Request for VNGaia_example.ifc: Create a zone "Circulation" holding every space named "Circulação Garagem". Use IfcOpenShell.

First a look at what the model holds.

```python
import ifcopenshell

model = ifcopenshell.open("VNGaia_example.ifc")
print(model.schema)
seen = {}
for space in model.by_type("IfcSpace"):
    seen[space.LongName] = seen.get(space.LongName, 0) + 1
for name, count in sorted(seen.items(), key=str):
    print(count, "x", name)
print("zones:", [z.Name for z in model.by_type("IfcZone")][:20])
```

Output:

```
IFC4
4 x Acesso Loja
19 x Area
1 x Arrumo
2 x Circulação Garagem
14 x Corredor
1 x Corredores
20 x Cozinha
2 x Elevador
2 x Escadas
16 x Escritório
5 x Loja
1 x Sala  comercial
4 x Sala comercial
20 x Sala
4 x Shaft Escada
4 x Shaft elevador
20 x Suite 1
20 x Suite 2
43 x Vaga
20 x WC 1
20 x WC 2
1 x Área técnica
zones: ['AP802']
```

```python
import ifcopenshell
import ifcopenshell.api.group
import ifcopenshell.api.root

model = ifcopenshell.open("VNGaia_example.ifc")

names = {"Circulação Garagem"}
spaces = [s for s in model.by_type("IfcSpace") if s.LongName in names]

zone = ifcopenshell.api.root.create_entity(model, ifc_class="IfcZone", name="Circulation")
ifcopenshell.api.group.assign_group(model, products=spaces, group=zone)
print(len(spaces), "spaces in", zone.Name)

model.write("VNGaia_example-out.ifc")
```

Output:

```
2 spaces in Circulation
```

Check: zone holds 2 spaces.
